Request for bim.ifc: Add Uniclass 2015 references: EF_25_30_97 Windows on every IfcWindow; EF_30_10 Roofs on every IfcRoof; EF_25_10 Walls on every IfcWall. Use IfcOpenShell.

First a look at what the model holds.

```python
import ifcopenshell

model = ifcopenshell.open("bim.ifc")
print(model.schema)
print("classifications:", [c.Name for c in model.by_type("IfcClassification")])
for ifc_class in ("IfcDoor", "IfcRoof", "IfcStair", "IfcWall", "IfcWindow"):
    print(ifc_class, len(model.by_type(ifc_class)))
```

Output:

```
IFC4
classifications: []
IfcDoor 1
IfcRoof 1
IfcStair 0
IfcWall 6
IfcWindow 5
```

```python
import ifcopenshell
import ifcopenshell.api.classification

model = ifcopenshell.open("bim.ifc")

system = ifcopenshell.api.classification.add_classification(model, classification="Uniclass 2015")

codes = {
    "IfcWindow": ("EF_25_30_97", "Windows"),
    "IfcRoof": ("EF_30_10", "Roofs"),
    "IfcWall": ("EF_25_10", "Walls"),
}
for ifc_class, (code, name) in codes.items():
    products = model.by_type(ifc_class)
    ifcopenshell.api.classification.add_reference(
        model, products=products, classification=system, identification=code, name=name
    )
    print(code, len(products))

model.write("bim_v2.ifc")
```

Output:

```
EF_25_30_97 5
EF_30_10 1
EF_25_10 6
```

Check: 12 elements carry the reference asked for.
